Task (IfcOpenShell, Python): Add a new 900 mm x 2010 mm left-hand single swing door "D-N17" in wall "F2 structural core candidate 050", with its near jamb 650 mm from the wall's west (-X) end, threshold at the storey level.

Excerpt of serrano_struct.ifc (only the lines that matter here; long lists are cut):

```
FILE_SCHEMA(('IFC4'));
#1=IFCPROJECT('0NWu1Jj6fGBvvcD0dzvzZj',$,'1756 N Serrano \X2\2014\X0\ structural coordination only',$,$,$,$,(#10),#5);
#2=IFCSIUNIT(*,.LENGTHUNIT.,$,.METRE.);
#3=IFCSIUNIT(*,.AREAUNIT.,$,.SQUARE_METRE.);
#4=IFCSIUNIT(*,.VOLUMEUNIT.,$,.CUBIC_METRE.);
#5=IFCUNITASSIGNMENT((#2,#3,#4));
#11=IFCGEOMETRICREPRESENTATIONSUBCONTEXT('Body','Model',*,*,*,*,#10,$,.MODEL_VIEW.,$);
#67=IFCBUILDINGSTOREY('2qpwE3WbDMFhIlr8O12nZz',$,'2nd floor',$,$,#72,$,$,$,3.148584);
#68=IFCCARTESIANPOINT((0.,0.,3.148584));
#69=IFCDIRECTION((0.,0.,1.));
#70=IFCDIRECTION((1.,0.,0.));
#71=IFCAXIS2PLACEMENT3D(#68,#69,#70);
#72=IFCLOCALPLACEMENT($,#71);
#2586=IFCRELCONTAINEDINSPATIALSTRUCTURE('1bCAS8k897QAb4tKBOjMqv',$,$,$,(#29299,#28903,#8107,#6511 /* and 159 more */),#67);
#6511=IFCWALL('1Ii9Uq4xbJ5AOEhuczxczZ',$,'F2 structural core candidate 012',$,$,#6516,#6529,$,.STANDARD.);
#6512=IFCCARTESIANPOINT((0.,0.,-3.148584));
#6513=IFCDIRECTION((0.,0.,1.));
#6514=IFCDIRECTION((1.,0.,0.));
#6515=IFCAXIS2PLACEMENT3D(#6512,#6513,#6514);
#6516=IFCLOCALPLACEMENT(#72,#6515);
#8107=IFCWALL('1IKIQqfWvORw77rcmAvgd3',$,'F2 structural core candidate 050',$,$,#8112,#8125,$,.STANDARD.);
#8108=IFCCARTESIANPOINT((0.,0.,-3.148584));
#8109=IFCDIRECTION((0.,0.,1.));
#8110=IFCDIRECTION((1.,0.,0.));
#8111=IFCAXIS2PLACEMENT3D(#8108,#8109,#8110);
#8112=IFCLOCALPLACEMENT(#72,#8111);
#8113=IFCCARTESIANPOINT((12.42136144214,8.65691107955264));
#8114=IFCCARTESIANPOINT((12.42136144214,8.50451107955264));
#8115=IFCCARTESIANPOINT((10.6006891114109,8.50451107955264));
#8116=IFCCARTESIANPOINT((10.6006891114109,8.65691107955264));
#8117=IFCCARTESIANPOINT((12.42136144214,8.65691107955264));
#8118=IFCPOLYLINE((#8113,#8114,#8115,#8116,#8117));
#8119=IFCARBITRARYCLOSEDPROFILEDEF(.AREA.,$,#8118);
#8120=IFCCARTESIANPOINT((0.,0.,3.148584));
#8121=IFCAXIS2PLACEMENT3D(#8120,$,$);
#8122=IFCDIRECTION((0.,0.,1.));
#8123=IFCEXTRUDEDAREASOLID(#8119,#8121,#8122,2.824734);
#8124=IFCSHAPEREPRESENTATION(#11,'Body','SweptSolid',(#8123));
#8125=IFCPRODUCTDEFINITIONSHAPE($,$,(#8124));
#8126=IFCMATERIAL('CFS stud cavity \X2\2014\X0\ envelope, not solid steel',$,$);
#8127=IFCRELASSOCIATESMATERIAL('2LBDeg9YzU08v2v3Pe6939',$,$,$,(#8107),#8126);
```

```python
import numpy as np
import ifcopenshell
import ifcopenshell.api.feature
import ifcopenshell.api.geometry
import ifcopenshell.api.root
import ifcopenshell.api.spatial
import ifcopenshell.geom
import ifcopenshell.util.element
import ifcopenshell.util.placement
import ifcopenshell.util.representation
import ifcopenshell.util.shape
import ifcopenshell.util.unit

model = ifcopenshell.open("serrano_struct.ifc")
unit_scale = ifcopenshell.util.unit.calculate_unit_scale(model)
settings = ifcopenshell.geom.settings()


def volume(element):
    """Net volume in cubic metres, openings subtracted."""
    shape = ifcopenshell.geom.create_shape(settings, element)
    return ifcopenshell.util.shape.get_volume(shape.geometry)


wall = model.by_guid("1IKIQqfWvORw77rcmAvgd3")
storey = ifcopenshell.util.element.get_container(wall, ifc_class="IfcBuildingStorey")
context = ifcopenshell.util.representation.get_context(model, "Model", "Body", "MODEL_VIEW")
before = volume(wall)

width, height, from_end, sill = 0.9, 2.01, 0.65, 0.0  # metres

# The wall runs along its own X axis, and the end named is its -X end.
wall_shape = ifcopenshell.geom.create_shape(settings, wall)
x, y, z = ifcopenshell.util.shape.get_vertices(wall_shape.geometry).T
start = x.min() + from_end
face, thickness = float(y.min()), float(y.max() - y.min())
wall_matrix = ifcopenshell.util.placement.get_local_placement(wall.ObjectPlacement)
level = ifcopenshell.util.placement.get_local_placement(storey.ObjectPlacement)[2, 3]


def in_wall(x, y):
    """Placement at x, y metres in the wall's axes, at sill height."""
    matrix = wall_matrix.copy()
    matrix[:, 3] = wall_matrix @ np.array([x / unit_scale, y / unit_scale, 0.0, 1.0])
    matrix[2, 3] = level + sill / unit_scale
    return matrix


# Opening: a box that overshoots both wall faces by 50 mm.
opening = ifcopenshell.api.root.create_entity(model, ifc_class="IfcOpeningElement", predefined_type="OPENING")
box = ifcopenshell.api.geometry.add_wall_representation(
    model, context=context, length=width, height=height, thickness=thickness + 0.1
)
ifcopenshell.api.geometry.assign_representation(model, product=opening, representation=box)
ifcopenshell.api.geometry.edit_object_placement(model, product=opening, matrix=in_wall(start, face - 0.05), is_si=False)
ifcopenshell.api.feature.add_feature(model, feature=opening, element=wall)

door = ifcopenshell.api.root.create_entity(model, ifc_class="IfcDoor", name="D-N17", predefined_type="DOOR")
door.OverallWidth, door.OverallHeight = width / unit_scale, height / unit_scale
door.OperationType = "SINGLE_SWING_LEFT"
body = ifcopenshell.api.geometry.add_door_representation(
    model,
    context=context,
    overall_width=door.OverallWidth,
    overall_height=door.OverallHeight,
    operation_type="SINGLE_SWING_LEFT",
    lining_properties={"LiningDepth": thickness / unit_scale, "ThresholdDepth": thickness / unit_scale},
)
ifcopenshell.api.geometry.assign_representation(model, product=door, representation=body)
ifcopenshell.api.spatial.assign_container(model, products=[door], relating_structure=storey)
ifcopenshell.api.feature.add_filling(model, opening=opening, element=door)

# The lining spans the wall, so the door starts at the wall face.
ifcopenshell.api.geometry.edit_object_placement(model, product=door, matrix=in_wall(start, face), is_si=False)

after = volume(wall)

print(f"wall volume {before:.3f} -> {after:.3f} m3")

model.write("serrano_struct_edited.ifc")
```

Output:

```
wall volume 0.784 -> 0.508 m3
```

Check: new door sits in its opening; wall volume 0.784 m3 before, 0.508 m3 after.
